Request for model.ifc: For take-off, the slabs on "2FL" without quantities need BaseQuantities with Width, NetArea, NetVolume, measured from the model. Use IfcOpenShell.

First a look at what the model holds.

```python
import ifcopenshell
import ifcopenshell.util.element
import ifcopenshell.util.unit

model = ifcopenshell.open("model.ifc")
print(model.schema)
for unit_type in ("LENGTHUNIT", "AREAUNIT", "VOLUMEUNIT"):
    print(unit_type, ifcopenshell.util.unit.calculate_unit_scale(model, unit_type))
storey = next(s for s in model.by_type("IfcBuildingStorey") if s.Name == "2FL")
slabs = [e for e in ifcopenshell.util.element.get_decomposition(storey) if e.is_a("IfcSlab")]
for e in sorted(slabs, key=lambda e: e.id()):
    print(e.id(), e.is_a(), e.Name, list(ifcopenshell.util.element.get_psets(e, qtos_only=True)), sep=" | ")
```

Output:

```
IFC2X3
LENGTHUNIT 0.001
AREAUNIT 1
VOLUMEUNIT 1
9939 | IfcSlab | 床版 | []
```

```python
import ifcopenshell
import ifcopenshell.api.pset
import ifcopenshell.geom
import ifcopenshell.util.element
import ifcopenshell.util.shape
import ifcopenshell.util.unit

model = ifcopenshell.open("model.ifc")
unit_scale = ifcopenshell.util.unit.calculate_unit_scale(model)
area_scale = ifcopenshell.util.unit.calculate_unit_scale(model, "AREAUNIT")
volume_scale = ifcopenshell.util.unit.calculate_unit_scale(model, "VOLUMEUNIT")
settings = ifcopenshell.geom.settings()

storey = next(s for s in model.by_type("IfcBuildingStorey") if s.Name == "2FL")
slabs = [e for e in ifcopenshell.util.element.get_decomposition(storey) if e.is_a("IfcSlab")]

for e in sorted(slabs, key=lambda e: e.id()):
    if ifcopenshell.util.element.get_psets(e, qtos_only=True, should_inherit=False):
        continue
    # Geometry comes back in metres, in the element's own axes.
    shape = ifcopenshell.geom.create_shape(settings, e)
    values = {
        "Width": ifcopenshell.util.shape.get_z(shape.geometry) / unit_scale,
        "NetArea": ifcopenshell.util.shape.get_footprint_area(shape.geometry) / area_scale,
        "NetVolume": ifcopenshell.util.shape.get_volume(shape.geometry) / volume_scale,
    }
    qto = ifcopenshell.api.pset.add_qto(model, product=e, name="BaseQuantities")
    ifcopenshell.api.pset.edit_qto(model, qto=qto, properties=values)
    print(e.id(), {k: round(v, 3) for k, v in values.items()})

model.write("model-out.ifc")
```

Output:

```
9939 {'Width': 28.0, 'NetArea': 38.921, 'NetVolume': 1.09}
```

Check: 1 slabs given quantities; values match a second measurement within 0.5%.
